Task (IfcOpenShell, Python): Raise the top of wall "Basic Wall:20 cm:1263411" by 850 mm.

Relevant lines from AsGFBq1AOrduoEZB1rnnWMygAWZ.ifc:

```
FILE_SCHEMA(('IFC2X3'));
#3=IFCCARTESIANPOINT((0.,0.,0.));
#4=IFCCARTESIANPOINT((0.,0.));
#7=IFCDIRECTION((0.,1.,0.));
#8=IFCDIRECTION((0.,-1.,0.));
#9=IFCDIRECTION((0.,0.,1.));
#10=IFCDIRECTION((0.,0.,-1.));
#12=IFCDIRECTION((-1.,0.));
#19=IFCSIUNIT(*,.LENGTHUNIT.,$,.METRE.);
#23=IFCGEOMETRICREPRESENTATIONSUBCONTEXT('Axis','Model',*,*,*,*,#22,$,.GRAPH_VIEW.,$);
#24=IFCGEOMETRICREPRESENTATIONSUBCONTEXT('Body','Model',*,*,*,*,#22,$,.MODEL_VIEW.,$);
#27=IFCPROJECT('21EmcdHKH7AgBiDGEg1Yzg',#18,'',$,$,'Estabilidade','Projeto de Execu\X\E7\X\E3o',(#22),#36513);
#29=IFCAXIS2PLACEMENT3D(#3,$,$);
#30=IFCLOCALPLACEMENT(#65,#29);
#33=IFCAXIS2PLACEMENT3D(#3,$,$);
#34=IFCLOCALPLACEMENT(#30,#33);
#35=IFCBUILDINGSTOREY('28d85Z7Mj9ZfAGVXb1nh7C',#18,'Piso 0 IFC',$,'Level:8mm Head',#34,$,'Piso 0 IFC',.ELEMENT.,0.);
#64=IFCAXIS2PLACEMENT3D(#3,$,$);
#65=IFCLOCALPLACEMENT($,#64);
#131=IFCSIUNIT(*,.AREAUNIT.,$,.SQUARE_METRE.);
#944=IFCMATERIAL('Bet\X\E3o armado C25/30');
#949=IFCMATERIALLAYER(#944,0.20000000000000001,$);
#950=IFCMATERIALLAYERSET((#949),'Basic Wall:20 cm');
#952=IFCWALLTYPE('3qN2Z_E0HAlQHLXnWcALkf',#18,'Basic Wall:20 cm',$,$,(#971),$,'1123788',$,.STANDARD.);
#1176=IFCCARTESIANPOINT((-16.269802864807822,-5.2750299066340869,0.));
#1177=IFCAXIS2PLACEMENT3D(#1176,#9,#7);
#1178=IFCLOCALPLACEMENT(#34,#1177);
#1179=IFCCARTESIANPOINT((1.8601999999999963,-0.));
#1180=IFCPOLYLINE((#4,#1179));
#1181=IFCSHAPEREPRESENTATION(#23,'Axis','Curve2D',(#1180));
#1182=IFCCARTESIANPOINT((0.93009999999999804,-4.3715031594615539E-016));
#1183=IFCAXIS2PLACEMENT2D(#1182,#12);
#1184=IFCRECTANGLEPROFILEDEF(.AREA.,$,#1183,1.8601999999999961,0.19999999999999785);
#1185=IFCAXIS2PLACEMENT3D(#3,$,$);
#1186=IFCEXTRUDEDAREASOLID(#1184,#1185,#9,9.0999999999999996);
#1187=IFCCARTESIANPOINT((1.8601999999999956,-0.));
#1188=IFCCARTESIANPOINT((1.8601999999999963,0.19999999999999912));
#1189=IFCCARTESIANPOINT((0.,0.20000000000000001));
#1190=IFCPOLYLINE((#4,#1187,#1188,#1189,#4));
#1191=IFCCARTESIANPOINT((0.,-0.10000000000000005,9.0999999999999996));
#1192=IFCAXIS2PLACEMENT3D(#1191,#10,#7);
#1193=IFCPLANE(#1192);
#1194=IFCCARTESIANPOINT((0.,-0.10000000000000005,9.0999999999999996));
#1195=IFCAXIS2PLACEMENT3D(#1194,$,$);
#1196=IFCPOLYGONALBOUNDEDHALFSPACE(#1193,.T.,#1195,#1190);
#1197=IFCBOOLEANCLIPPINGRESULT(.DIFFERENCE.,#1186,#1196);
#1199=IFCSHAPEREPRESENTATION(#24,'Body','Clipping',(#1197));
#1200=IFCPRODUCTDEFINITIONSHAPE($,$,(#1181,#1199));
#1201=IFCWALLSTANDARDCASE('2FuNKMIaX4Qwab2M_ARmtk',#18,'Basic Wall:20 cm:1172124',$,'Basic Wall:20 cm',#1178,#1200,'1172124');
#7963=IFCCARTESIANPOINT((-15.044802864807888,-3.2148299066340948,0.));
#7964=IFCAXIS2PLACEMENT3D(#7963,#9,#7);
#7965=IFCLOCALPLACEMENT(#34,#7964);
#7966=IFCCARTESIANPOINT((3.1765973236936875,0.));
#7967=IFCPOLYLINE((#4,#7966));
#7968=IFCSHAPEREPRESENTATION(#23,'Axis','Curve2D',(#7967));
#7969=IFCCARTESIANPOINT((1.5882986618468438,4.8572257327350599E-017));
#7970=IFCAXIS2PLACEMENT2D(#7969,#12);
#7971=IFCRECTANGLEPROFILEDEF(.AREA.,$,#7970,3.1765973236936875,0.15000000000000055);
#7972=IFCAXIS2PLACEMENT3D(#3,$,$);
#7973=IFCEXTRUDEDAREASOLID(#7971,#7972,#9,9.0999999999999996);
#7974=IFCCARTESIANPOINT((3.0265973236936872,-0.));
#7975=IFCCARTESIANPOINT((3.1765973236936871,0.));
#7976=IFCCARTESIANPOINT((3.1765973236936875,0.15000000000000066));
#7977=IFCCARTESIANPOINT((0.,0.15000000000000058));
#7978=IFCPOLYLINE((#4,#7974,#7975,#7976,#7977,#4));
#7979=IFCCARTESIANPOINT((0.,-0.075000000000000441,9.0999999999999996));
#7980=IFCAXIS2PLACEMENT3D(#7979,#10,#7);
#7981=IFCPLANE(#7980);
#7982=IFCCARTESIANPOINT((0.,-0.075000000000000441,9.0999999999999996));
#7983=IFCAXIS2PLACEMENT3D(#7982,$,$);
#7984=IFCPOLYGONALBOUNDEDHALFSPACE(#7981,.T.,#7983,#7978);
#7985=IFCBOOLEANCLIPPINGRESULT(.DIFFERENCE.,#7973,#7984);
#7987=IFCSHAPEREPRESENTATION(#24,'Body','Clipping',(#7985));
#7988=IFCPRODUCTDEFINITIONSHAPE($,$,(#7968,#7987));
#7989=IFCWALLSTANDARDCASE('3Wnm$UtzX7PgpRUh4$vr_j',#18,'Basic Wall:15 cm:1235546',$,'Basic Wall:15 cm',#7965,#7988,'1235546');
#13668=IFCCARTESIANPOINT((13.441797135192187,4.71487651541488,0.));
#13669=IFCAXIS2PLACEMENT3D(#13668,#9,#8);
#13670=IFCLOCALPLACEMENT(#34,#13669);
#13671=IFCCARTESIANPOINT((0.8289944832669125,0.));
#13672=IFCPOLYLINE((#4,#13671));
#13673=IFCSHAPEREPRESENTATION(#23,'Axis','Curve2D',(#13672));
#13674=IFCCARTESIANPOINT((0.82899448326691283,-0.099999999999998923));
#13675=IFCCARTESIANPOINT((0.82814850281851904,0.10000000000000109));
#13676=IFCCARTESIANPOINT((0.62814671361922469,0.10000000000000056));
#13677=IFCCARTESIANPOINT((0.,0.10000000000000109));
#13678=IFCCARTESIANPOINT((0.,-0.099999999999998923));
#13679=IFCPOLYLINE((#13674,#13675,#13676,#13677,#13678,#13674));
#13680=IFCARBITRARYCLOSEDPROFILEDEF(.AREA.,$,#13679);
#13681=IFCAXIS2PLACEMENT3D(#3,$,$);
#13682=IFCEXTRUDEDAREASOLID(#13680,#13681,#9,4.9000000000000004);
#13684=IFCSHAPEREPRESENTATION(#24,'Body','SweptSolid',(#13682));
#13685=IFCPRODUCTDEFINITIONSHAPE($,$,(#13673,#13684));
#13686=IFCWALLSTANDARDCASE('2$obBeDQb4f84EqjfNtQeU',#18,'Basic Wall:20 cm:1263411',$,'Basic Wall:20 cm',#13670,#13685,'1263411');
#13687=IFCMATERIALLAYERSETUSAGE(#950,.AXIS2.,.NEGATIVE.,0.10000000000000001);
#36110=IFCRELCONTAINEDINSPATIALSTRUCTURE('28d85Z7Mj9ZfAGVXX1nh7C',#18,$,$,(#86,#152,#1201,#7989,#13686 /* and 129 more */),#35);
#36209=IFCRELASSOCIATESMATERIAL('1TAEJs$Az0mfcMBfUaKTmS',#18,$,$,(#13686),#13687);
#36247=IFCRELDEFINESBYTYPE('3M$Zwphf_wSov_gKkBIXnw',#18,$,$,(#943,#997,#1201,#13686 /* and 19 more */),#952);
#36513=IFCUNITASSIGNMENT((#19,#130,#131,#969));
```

```python
import ifcopenshell
import ifcopenshell.geom
import ifcopenshell.util.representation
import ifcopenshell.util.shape

model = ifcopenshell.open("AsGFBq1AOrduoEZB1rnnWMygAWZ.ifc")
settings = ifcopenshell.geom.settings()


def volume(element):
    """Net volume in cubic metres, openings subtracted."""
    shape = ifcopenshell.geom.create_shape(settings, element)
    return ifcopenshell.util.shape.get_volume(shape.geometry)


wall = model.by_id(13686)
before = volume(wall)

body = ifcopenshell.util.representation.get_representation(wall, "Model", "Body")
solid = body.Items[0]
old_height = solid.Depth
solid.Depth += 0.85
after = volume(wall)

print(f"height {old_height:g} -> {solid.Depth:g}, volume {before:.3f} -> {after:.3f} m3")

model.write("AsGFBq1AOrduoEZB1rnnWMygAWZ_edited.ifc")
```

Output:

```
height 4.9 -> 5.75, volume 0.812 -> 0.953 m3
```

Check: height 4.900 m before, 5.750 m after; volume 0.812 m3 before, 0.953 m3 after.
